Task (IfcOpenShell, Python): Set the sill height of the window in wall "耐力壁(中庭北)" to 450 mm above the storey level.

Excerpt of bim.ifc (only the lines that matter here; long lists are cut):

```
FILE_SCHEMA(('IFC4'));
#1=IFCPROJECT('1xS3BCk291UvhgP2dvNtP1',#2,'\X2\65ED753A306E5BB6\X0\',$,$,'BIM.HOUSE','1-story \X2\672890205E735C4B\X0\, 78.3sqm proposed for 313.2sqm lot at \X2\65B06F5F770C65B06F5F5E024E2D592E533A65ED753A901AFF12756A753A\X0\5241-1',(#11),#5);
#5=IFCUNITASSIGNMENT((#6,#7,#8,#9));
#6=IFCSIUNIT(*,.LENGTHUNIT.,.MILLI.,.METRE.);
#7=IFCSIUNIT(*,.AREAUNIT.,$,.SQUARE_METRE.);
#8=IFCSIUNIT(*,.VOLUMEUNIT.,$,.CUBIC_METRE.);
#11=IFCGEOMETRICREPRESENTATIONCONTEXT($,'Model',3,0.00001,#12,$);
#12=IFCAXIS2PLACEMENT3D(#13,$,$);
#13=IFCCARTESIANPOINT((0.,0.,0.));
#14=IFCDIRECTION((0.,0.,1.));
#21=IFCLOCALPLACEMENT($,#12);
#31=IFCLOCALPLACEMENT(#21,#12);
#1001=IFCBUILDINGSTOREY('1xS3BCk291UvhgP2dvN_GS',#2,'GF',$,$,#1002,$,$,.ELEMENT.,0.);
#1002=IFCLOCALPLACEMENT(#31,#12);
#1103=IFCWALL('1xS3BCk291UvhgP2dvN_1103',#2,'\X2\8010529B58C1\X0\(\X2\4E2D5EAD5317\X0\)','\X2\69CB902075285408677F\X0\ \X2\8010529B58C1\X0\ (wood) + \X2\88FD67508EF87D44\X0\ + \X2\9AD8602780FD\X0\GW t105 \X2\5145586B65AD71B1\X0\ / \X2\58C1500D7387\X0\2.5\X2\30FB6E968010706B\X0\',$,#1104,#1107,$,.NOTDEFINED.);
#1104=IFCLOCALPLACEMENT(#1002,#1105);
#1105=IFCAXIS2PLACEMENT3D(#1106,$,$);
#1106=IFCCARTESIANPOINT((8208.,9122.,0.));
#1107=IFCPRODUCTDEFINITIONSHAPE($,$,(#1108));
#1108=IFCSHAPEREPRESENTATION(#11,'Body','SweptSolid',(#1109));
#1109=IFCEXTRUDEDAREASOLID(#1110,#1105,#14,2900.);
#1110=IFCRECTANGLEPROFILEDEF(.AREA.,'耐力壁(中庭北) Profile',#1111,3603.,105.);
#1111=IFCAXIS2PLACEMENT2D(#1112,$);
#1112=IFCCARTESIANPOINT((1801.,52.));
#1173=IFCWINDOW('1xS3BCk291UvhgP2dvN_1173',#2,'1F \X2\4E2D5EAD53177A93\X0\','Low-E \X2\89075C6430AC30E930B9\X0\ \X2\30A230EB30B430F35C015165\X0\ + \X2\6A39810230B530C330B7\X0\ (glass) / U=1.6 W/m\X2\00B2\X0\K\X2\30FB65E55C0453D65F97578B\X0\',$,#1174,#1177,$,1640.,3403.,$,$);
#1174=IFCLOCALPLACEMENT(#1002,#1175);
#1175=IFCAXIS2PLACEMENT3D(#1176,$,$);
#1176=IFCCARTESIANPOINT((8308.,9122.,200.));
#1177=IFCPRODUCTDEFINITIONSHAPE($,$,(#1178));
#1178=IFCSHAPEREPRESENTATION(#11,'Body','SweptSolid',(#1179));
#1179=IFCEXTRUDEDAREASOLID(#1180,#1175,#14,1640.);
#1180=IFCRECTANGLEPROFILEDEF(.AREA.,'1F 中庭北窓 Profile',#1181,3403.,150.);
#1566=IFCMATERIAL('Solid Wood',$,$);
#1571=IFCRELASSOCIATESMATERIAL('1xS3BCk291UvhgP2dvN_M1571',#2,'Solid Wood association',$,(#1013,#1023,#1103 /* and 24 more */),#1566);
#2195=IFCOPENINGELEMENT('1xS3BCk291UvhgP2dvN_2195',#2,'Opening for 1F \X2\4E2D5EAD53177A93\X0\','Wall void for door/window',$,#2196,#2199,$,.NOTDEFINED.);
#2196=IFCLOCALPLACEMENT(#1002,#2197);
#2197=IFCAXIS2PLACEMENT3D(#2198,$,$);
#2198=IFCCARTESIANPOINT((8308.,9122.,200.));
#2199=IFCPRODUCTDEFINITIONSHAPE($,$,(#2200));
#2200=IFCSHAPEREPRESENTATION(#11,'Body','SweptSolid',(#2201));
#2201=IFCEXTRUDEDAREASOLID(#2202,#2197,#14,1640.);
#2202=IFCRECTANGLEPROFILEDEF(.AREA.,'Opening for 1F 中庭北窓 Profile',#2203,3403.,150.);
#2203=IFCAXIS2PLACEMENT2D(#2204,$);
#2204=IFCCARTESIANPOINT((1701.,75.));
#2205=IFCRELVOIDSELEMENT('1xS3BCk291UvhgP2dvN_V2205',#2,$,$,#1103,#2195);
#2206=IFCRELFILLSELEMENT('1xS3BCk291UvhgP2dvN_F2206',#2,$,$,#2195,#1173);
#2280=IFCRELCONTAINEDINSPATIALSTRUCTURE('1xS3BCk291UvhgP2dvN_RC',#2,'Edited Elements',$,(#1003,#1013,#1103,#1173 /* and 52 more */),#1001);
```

```python
import numpy as np
import ifcopenshell
import ifcopenshell.api.geometry
import ifcopenshell.geom
import ifcopenshell.util.element
import ifcopenshell.util.placement
import ifcopenshell.util.shape
import ifcopenshell.util.unit

model = ifcopenshell.open("bim.ifc")
unit_scale = ifcopenshell.util.unit.calculate_unit_scale(model)

window = model.by_id(1173)
opening = window.FillsVoids[0].RelatingOpeningElement
storey = ifcopenshell.util.element.get_container(window, ifc_class="IfcBuildingStorey")
level = ifcopenshell.util.placement.get_local_placement(storey.ObjectPlacement)[2, 3]

# The opening's origin need not be at the sill, so measure its lowest point.
shape = ifcopenshell.geom.create_shape(ifcopenshell.geom.settings(), opening)
bottom = ifcopenshell.util.shape.get_shape_bottom_elevation(shape, shape.geometry) / unit_scale
dz = level + 450.0 - bottom

shift = np.array([0.0, 0.0, dz])
# The window is not placed relative to its opening, so move both.
for product in (opening, window):
    matrix = ifcopenshell.util.placement.get_local_placement(product.ObjectPlacement)
    matrix[:3, 3] += shift
    ifcopenshell.api.geometry.edit_object_placement(model, product=product, matrix=matrix, is_si=False)

print(f"moved by {dz * unit_scale:+.3f} m")

model.write("bim_v2.ifc")
```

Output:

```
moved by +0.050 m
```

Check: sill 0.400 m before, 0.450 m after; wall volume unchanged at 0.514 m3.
